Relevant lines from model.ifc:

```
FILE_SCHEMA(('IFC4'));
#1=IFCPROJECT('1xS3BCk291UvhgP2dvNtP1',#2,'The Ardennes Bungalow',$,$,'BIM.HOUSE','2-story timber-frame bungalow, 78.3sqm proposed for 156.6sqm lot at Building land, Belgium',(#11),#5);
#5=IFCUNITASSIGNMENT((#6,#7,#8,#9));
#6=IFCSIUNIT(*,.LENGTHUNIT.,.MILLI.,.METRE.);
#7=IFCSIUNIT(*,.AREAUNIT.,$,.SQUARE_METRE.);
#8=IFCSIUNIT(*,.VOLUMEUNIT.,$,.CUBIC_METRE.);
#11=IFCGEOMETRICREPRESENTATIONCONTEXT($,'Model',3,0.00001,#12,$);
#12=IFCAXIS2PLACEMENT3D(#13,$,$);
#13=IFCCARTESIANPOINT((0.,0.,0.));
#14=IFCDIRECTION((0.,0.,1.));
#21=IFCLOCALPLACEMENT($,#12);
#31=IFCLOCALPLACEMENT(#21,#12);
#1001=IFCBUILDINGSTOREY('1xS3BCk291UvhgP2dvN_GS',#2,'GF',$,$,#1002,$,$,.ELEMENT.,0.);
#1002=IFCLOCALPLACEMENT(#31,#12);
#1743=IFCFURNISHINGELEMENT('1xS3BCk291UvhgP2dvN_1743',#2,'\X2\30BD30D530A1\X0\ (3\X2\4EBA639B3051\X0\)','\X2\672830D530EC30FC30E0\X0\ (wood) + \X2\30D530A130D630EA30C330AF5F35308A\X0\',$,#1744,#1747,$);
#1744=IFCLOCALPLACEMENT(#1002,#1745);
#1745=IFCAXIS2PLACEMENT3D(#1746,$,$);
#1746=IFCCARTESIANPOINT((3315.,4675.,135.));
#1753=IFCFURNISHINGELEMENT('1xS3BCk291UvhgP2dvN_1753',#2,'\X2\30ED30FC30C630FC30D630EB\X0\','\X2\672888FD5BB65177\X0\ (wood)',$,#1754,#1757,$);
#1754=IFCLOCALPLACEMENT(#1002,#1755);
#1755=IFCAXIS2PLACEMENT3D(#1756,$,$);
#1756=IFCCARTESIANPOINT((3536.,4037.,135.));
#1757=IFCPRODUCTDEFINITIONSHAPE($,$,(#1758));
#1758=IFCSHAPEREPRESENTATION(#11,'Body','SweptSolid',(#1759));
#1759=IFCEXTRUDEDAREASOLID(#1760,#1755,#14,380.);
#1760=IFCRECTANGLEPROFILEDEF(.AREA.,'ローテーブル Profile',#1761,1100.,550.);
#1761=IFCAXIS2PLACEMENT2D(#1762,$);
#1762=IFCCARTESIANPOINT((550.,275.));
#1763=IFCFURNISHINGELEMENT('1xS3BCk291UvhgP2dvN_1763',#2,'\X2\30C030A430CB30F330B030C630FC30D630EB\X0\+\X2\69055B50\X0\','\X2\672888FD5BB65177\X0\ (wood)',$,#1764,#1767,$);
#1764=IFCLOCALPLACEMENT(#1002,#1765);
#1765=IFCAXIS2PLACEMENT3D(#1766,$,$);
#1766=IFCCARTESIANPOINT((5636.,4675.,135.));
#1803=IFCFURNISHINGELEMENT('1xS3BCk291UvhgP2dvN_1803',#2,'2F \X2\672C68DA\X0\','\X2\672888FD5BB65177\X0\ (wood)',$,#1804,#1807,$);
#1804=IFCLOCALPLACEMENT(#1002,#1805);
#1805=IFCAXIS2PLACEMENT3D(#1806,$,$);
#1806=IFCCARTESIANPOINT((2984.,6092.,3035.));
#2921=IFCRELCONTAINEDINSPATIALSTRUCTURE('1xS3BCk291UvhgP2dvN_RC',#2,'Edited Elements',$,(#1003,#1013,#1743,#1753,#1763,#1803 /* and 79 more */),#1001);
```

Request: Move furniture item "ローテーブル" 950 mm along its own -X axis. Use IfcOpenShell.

```python
import ifcopenshell
import ifcopenshell.api.geometry
import ifcopenshell.util.placement
import ifcopenshell.util.unit

model = ifcopenshell.open("model.ifc")
unit_scale = ifcopenshell.util.unit.calculate_unit_scale(model)

item = model.by_guid("1xS3BCk291UvhgP2dvN_1753")
matrix = ifcopenshell.util.placement.get_local_placement(item.ObjectPlacement)
matrix[:3, 3] -= matrix[:3, 0] * 0.95 / unit_scale
ifcopenshell.api.geometry.edit_object_placement(model, product=item, matrix=matrix, is_si=False)

print(ifcopenshell.util.placement.get_local_placement(item.ObjectPlacement).round(3) + 0.0)

model.write("model-out.ifc")
```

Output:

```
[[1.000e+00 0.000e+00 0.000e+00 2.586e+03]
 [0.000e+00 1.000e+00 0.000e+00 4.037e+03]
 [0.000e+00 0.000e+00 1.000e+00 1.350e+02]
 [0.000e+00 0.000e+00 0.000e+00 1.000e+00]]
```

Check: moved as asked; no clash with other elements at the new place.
